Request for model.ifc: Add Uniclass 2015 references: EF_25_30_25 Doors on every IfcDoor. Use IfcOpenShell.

First a look at what the model holds.

```python
import ifcopenshell

model = ifcopenshell.open("model.ifc")
print(model.schema)
print("classifications:", [c.Name for c in model.by_type("IfcClassification")])
for ifc_class in ("IfcDoor", "IfcRoof", "IfcStair", "IfcWall", "IfcWindow"):
    print(ifc_class, len(model.by_type(ifc_class)))
```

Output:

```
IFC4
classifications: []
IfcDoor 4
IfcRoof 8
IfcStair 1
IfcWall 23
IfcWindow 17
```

```python
import ifcopenshell
import ifcopenshell.api.classification

model = ifcopenshell.open("model.ifc")

system = ifcopenshell.api.classification.add_classification(model, classification="Uniclass 2015")

codes = {
    "IfcDoor": ("EF_25_30_25", "Doors"),
}
for ifc_class, (code, name) in codes.items():
    products = model.by_type(ifc_class)
    ifcopenshell.api.classification.add_reference(
        model, products=products, classification=system, identification=code, name=name
    )
    print(code, len(products))

model.write("model_updated.ifc")
```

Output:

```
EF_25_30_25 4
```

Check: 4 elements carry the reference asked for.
